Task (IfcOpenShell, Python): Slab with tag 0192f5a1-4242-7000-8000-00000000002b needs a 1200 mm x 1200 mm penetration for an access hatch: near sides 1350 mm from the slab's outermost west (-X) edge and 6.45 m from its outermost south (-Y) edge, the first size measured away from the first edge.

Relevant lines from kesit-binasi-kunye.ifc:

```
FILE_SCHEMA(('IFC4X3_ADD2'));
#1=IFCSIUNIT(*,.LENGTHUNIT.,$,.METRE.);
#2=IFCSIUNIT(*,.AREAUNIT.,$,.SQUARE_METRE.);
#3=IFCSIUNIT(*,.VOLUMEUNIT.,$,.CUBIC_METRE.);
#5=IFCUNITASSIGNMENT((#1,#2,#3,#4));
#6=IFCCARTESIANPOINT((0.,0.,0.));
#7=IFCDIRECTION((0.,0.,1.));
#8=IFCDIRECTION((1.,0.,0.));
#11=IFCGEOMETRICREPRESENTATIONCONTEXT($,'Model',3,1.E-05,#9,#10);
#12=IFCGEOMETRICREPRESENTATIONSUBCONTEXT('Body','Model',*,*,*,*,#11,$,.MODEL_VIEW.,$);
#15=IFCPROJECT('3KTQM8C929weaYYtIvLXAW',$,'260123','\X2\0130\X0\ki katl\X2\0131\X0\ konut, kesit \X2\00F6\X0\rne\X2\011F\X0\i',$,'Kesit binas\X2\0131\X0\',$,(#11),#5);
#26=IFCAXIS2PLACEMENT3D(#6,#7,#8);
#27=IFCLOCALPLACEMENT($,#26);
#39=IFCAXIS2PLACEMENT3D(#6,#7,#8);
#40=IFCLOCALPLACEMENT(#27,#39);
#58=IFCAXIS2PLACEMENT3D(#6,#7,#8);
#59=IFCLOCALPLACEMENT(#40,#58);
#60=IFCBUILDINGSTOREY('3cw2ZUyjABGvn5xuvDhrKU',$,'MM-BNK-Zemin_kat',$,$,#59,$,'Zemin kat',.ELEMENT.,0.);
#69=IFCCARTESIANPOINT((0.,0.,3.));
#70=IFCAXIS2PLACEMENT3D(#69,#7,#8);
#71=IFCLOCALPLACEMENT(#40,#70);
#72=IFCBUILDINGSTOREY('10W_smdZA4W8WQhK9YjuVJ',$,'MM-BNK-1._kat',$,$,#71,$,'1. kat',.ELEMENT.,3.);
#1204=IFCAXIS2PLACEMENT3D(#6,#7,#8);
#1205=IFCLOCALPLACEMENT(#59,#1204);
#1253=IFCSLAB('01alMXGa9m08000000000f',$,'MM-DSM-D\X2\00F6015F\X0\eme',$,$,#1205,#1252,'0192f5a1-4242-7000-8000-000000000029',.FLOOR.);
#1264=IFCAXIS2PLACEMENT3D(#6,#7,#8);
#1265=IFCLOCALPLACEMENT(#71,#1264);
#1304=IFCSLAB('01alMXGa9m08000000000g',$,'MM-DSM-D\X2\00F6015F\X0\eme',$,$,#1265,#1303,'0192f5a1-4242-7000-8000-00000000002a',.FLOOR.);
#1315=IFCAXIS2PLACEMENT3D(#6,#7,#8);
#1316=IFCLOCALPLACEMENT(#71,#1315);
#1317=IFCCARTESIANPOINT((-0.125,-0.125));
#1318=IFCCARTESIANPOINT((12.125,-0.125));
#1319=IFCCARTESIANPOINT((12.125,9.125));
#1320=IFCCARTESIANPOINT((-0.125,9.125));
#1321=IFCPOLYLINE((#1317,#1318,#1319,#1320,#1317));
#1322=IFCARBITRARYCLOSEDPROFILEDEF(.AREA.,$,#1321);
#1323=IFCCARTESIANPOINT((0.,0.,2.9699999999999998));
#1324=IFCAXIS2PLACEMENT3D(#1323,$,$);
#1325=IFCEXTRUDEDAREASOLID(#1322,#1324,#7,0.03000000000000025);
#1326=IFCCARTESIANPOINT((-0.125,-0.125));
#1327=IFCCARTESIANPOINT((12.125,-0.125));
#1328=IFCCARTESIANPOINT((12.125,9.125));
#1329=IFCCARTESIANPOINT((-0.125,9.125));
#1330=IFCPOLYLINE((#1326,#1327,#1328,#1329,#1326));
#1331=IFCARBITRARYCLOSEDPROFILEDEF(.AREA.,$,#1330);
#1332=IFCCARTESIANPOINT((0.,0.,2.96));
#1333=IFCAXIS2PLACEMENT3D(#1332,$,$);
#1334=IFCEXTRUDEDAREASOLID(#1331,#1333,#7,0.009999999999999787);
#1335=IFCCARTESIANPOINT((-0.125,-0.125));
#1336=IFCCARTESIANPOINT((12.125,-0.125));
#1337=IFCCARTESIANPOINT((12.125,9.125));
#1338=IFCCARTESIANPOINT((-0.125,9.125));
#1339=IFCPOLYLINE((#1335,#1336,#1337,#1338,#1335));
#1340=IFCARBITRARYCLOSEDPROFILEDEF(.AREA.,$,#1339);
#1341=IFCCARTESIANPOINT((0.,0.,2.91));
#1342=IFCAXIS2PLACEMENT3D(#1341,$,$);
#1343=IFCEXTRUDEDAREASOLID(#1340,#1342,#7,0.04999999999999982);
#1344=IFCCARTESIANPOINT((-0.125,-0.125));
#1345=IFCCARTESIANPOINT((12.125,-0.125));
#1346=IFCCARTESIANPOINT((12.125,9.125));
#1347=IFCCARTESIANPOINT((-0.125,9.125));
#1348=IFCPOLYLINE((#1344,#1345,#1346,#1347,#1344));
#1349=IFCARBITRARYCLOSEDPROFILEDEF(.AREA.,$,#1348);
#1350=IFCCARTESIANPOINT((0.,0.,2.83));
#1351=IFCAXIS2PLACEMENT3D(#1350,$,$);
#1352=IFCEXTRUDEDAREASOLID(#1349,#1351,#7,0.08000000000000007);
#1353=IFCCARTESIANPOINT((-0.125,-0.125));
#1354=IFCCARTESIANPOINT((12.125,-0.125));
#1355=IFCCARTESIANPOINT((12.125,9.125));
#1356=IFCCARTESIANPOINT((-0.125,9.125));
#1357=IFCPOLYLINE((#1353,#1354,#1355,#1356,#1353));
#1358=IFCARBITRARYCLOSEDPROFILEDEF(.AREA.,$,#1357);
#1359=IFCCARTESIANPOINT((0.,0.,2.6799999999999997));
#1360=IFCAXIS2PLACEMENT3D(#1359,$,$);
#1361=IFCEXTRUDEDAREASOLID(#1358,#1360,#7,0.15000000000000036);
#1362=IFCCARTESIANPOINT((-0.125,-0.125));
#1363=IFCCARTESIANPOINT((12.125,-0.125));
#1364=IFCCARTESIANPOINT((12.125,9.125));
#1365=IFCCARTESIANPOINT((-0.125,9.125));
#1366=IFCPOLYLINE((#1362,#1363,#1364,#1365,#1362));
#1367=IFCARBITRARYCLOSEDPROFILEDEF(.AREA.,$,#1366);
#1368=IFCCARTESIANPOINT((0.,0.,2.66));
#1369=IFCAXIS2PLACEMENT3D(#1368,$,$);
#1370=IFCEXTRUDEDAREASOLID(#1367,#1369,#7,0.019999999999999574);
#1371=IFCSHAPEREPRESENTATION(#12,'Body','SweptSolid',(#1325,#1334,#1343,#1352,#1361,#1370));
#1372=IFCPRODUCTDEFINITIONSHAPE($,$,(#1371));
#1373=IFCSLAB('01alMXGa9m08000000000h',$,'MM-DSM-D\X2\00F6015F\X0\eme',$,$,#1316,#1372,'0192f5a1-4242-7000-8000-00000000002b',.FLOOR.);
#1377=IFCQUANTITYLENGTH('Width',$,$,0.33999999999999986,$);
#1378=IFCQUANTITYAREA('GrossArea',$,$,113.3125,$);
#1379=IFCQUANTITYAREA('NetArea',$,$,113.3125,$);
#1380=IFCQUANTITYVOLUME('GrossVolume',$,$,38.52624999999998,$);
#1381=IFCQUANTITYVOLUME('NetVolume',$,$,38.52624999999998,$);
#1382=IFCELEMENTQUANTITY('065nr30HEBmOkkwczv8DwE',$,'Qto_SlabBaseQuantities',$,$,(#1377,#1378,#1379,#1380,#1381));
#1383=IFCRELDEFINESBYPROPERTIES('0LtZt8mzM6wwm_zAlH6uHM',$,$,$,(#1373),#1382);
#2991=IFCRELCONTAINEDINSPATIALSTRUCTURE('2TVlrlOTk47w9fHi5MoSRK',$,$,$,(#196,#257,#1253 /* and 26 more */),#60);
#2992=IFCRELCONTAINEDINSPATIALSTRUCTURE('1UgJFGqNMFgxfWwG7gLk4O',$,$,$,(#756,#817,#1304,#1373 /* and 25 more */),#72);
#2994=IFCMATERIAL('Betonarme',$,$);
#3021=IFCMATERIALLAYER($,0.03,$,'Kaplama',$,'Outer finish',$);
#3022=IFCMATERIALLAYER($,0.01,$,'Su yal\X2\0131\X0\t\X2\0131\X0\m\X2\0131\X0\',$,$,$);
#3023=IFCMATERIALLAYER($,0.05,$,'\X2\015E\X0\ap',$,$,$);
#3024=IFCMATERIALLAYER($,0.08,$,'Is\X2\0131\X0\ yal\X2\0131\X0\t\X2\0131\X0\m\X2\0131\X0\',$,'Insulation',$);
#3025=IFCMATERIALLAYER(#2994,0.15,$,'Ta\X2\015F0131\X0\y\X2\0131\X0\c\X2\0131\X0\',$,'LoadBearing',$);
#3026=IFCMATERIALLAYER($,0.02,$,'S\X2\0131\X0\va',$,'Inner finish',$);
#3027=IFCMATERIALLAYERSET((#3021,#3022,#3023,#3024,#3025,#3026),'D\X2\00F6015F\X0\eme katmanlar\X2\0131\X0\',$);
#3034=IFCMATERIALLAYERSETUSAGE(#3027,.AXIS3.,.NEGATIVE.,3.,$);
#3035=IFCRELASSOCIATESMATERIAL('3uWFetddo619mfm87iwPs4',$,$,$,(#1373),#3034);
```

```python
import numpy as np
import ifcopenshell
import ifcopenshell.api.feature
import ifcopenshell.api.geometry
import ifcopenshell.api.pset
import ifcopenshell.api.root
import ifcopenshell.geom
import ifcopenshell.util.element
import ifcopenshell.util.placement
import ifcopenshell.util.representation
import ifcopenshell.util.shape
import ifcopenshell.util.unit

model = ifcopenshell.open("kesit-binasi-kunye.ifc")
unit_scale = ifcopenshell.util.unit.calculate_unit_scale(model)
area_scale = ifcopenshell.util.unit.calculate_unit_scale(model, "AREAUNIT")
volume_scale = ifcopenshell.util.unit.calculate_unit_scale(model, "VOLUMEUNIT")
settings = ifcopenshell.geom.settings()


def volume(element):
    """Net volume in cubic metres, openings subtracted."""
    shape = ifcopenshell.geom.create_shape(settings, element)
    return ifcopenshell.util.shape.get_volume(shape.geometry)


slab = model.by_guid("01alMXGa9m08000000000h")
before = volume(slab)

# Extent in the slab's own axes, in metres. The edges named are its -X and -Y sides.
slab_shape = ifcopenshell.geom.create_shape(settings, slab)
vertices = ifcopenshell.util.shape.get_vertices(slab_shape.geometry)
x_min, y_min, bottom = vertices.min(axis=0)
top = vertices[:, 2].max()

opening = ifcopenshell.api.root.create_entity(model, ifc_class="IfcOpeningElement", name="Access hatch opening", predefined_type="OPENING")
context = ifcopenshell.util.representation.get_context(model, "Model", "Body", "MODEL_VIEW")
width, depth = 1.2, 1.2
outline = [(0.0, 0.0), (width, 0.0), (width, depth), (0.0, depth), (0.0, 0.0)]
# Overshoot both faces by 50 mm so the cut is clean.
shape = ifcopenshell.api.geometry.add_slab_representation(
    model, context=context, depth=top - bottom + 0.1, polyline=outline
)
ifcopenshell.api.geometry.assign_representation(model, product=opening, representation=shape)

matrix = ifcopenshell.util.placement.get_local_placement(slab.ObjectPlacement)
matrix[:, 3] = matrix @ np.append(np.array([x_min + 1.35, y_min + 6.45, bottom - 0.05]) / unit_scale, 1.0)
ifcopenshell.api.geometry.edit_object_placement(model, product=opening, matrix=matrix, is_si=False)
ifcopenshell.api.feature.add_feature(model, feature=opening, element=slab)

after = volume(slab)

# Update the slab's stored quantities.
qto = model.by_id(ifcopenshell.util.element.get_pset(slab, "Qto_SlabBaseQuantities", should_inherit=False)["id"])
ifcopenshell.api.pset.edit_qto(model, qto=qto, properties={
    "NetArea": after / (top - bottom) / area_scale,
    "NetVolume": after / volume_scale,
})

print(f"slab volume {before:.3f} -> {after:.3f} m3")

model.write("kesit-binasi-kunye_rev.ifc")
```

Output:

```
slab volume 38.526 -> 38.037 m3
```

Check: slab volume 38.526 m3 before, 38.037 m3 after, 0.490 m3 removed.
